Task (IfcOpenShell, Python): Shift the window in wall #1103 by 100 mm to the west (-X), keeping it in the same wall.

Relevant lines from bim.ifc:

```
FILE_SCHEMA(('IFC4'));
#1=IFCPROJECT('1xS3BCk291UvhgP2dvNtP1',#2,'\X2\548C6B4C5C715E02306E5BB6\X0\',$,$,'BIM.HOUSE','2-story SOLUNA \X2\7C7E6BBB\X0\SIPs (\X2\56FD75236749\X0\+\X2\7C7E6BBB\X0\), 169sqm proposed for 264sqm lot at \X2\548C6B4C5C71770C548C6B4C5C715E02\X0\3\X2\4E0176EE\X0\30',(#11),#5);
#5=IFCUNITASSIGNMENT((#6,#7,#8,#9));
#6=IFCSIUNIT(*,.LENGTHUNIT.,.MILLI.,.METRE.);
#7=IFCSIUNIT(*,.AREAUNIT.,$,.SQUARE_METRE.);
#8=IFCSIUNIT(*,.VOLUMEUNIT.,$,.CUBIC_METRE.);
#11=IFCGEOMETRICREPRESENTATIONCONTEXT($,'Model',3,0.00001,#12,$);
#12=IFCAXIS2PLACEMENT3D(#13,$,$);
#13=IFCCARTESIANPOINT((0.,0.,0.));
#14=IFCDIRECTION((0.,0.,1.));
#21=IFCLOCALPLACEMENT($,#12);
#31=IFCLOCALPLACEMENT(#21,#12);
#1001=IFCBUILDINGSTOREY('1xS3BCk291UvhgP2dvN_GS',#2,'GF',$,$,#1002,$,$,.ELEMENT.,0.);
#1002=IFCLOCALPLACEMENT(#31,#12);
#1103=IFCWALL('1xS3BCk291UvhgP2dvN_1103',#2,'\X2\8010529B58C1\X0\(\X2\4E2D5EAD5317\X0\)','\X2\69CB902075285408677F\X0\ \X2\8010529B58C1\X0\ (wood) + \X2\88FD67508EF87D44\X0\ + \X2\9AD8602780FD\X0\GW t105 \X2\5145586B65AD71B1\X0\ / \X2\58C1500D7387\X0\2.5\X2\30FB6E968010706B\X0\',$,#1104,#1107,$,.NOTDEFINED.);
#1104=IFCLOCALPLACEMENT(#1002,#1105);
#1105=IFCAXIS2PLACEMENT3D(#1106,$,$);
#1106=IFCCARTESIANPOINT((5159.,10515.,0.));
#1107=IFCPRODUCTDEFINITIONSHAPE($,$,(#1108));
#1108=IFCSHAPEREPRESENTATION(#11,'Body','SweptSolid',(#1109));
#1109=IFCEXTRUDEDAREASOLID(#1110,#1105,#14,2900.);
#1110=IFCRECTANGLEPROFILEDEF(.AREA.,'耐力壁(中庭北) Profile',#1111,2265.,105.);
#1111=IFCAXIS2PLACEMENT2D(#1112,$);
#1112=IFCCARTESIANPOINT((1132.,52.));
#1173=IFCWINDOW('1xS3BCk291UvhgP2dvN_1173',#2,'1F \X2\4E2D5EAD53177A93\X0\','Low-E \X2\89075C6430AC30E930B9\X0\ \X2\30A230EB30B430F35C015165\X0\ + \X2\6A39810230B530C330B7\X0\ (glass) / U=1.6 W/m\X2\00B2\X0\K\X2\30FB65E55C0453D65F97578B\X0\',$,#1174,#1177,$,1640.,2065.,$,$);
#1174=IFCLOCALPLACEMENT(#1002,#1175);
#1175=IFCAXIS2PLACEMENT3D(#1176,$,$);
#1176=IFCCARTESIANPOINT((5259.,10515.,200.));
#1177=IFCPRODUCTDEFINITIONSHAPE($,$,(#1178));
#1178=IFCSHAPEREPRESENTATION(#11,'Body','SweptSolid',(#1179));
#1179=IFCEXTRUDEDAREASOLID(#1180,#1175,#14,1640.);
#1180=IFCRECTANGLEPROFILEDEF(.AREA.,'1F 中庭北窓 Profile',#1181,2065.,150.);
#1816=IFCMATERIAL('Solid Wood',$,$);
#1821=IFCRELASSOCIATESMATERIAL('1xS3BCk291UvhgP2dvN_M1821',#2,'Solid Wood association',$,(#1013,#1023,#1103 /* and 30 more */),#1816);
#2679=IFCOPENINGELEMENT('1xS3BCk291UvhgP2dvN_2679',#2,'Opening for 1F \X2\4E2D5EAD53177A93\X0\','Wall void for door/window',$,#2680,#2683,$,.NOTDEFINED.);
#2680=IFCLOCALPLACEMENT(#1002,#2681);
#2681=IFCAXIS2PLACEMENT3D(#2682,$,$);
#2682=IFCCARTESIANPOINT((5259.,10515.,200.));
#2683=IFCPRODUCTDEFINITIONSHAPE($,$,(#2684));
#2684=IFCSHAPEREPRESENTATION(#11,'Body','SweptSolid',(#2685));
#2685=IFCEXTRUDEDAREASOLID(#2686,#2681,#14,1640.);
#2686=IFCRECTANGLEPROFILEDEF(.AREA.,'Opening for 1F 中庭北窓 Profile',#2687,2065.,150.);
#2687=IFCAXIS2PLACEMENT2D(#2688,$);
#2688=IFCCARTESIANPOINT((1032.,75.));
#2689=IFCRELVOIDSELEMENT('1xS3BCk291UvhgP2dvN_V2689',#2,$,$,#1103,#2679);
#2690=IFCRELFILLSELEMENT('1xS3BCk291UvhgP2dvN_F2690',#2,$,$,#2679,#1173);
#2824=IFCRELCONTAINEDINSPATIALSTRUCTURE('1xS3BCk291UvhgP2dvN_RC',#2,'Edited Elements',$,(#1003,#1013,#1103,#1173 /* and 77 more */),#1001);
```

```python
import ifcopenshell
import ifcopenshell.api.geometry
import ifcopenshell.util.placement

model = ifcopenshell.open("bim.ifc")

window = model.by_id(1173)
opening = window.FillsVoids[0].RelatingOpeningElement
wall = opening.VoidsElements[0].RelatingBuildingElement

wall_matrix = ifcopenshell.util.placement.get_local_placement(wall.ObjectPlacement)
shift = wall_matrix[:3, 0] * -100.0
before = ifcopenshell.util.placement.get_local_placement(window.ObjectPlacement)[:3, 3].copy()

# The window is not placed relative to its opening, so move both.
for product in (opening, window):
    matrix = ifcopenshell.util.placement.get_local_placement(product.ObjectPlacement)
    matrix[:3, 3] += shift
    ifcopenshell.api.geometry.edit_object_placement(model, product=product, matrix=matrix, is_si=False)

after = ifcopenshell.util.placement.get_local_placement(window.ObjectPlacement)[:3, 3]
print("window moved by", (after - before).round(3) + 0.0)

model.write("bim_v2.ifc")
```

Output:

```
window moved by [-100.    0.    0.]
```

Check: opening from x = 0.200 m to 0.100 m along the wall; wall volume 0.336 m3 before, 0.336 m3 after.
